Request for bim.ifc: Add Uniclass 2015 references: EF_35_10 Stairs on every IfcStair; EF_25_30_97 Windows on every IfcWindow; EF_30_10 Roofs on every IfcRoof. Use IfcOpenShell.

First a look at what the model holds.

```python
import ifcopenshell

model = ifcopenshell.open("bim.ifc")
print(model.schema)
print("classifications:", [c.Name for c in model.by_type("IfcClassification")])
for ifc_class in ("IfcDoor", "IfcRoof", "IfcStair", "IfcWall", "IfcWindow"):
    print(ifc_class, len(model.by_type(ifc_class)))
```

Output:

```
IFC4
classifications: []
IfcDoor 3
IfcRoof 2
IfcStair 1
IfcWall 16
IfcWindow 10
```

```python
import ifcopenshell
import ifcopenshell.api.classification

model = ifcopenshell.open("bim.ifc")

system = ifcopenshell.api.classification.add_classification(model, classification="Uniclass 2015")

codes = {
    "IfcStair": ("EF_35_10", "Stairs"),
    "IfcWindow": ("EF_25_30_97", "Windows"),
    "IfcRoof": ("EF_30_10", "Roofs"),
}
for ifc_class, (code, name) in codes.items():
    products = model.by_type(ifc_class)
    ifcopenshell.api.classification.add_reference(
        model, products=products, classification=system, identification=code, name=name
    )
    print(code, len(products))

model.write("bim_rev.ifc")
```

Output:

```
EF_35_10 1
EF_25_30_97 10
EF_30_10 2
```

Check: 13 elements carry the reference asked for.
